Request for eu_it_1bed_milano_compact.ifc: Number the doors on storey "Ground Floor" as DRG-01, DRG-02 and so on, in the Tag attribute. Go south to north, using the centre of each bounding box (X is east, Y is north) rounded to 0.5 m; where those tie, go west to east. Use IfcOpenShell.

First a look at what the model holds.

```python
import ifcopenshell
import ifcopenshell.util.element
import ifcopenshell.util.placement

model = ifcopenshell.open("eu_it_1bed_milano_compact.ifc")
print(model.schema)
storey = next(s for s in model.by_type("IfcBuildingStorey") if s.Name == "Ground Floor")
doors = [e for e in ifcopenshell.util.element.get_decomposition(storey) if e.is_a("IfcDoor")]
for e in sorted(doors, key=lambda e: e.id()):
    origin = ifcopenshell.util.placement.get_local_placement(e.ObjectPlacement)[:3, 3]
    print(e.id(), e.Tag, e.Name, origin.round(2) + 0.0, sep=" | ")
```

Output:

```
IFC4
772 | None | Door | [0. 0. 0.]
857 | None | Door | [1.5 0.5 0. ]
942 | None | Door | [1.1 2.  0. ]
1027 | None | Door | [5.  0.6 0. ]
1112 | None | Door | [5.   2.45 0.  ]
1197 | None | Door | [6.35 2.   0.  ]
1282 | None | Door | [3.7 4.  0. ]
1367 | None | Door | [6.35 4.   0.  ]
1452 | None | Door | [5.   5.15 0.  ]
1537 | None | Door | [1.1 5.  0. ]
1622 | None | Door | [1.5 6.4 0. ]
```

```python
import ifcopenshell
import ifcopenshell.geom
import ifcopenshell.util.element
import ifcopenshell.util.shape

model = ifcopenshell.open("eu_it_1bed_milano_compact.ifc")
settings = ifcopenshell.geom.settings()
settings.set("use-world-coords", True)


def centre(element):
    shape = ifcopenshell.geom.create_shape(settings, element)
    return ifcopenshell.util.shape.get_bbox_centroid(shape.geometry)


storey = next(s for s in model.by_type("IfcBuildingStorey") if s.Name == "Ground Floor")
doors = [e for e in ifcopenshell.util.element.get_decomposition(storey) if e.is_a("IfcDoor")]

# Insertion points can sit at a corner or the storey origin, so sort by the geometry (in metres).
centres = {e: centre(e) for e in doors}
doors.sort(key=lambda e: (round(centres[e][1] / 0.5), centres[e][0]))

for i, e in enumerate(doors, start=1):
    number = f"DRG-{i:02d}"
    e.Tag = number
    print(e.id(), number)

model.write("eu_it_1bed_milano_compact_updated.ifc")
```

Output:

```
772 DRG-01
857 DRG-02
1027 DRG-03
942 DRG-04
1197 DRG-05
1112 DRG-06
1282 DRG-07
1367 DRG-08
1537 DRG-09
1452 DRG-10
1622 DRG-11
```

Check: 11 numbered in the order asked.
